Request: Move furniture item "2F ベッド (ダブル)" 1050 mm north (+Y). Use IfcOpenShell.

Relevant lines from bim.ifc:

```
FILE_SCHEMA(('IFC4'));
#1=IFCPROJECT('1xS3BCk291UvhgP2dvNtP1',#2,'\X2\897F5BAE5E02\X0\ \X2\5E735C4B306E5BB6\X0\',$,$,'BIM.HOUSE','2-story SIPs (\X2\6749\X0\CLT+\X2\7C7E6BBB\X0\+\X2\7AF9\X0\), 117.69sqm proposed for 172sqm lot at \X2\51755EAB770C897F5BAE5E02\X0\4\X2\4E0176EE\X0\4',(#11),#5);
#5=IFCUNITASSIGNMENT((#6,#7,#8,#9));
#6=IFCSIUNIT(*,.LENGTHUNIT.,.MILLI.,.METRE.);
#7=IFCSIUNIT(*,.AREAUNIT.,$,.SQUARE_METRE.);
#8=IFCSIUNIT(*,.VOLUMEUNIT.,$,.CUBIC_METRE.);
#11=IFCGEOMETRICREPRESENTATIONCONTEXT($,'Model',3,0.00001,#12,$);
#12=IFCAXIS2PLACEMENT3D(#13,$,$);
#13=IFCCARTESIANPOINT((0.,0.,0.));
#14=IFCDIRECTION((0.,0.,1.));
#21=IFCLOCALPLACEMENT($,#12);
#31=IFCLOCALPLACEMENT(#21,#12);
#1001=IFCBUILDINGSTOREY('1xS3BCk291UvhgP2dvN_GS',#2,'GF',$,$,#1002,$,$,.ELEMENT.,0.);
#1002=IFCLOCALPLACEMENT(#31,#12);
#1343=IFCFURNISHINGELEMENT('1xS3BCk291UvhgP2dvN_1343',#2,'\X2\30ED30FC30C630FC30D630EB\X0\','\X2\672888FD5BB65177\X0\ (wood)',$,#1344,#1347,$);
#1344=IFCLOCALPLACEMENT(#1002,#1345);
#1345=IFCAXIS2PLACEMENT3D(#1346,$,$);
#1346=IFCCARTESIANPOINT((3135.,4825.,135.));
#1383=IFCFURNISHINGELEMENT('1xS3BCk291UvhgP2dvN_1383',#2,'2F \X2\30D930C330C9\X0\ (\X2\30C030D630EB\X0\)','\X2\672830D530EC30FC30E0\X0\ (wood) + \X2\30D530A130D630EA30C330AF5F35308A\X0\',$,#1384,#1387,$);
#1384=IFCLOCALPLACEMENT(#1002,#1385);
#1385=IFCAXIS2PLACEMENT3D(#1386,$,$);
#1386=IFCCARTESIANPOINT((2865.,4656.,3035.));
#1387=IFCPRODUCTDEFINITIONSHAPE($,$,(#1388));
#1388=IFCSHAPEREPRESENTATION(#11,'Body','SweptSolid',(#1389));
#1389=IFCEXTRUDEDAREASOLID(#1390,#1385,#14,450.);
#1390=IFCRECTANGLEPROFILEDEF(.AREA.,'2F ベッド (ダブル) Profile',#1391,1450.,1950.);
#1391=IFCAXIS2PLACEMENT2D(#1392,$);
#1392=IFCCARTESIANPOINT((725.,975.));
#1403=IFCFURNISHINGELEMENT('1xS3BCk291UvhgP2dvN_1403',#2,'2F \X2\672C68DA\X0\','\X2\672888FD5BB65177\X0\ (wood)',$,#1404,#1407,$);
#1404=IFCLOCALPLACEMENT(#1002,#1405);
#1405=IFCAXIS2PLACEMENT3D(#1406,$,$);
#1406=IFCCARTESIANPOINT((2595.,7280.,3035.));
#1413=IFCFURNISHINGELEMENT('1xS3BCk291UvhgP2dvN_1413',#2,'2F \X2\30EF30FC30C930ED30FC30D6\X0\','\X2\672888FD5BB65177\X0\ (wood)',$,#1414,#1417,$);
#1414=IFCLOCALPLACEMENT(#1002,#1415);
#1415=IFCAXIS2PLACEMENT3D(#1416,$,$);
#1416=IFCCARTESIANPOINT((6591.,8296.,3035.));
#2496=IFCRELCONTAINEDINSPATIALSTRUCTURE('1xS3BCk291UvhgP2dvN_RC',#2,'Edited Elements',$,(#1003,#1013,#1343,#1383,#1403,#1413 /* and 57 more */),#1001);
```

```python
import ifcopenshell
import ifcopenshell.api.geometry
import ifcopenshell.util.placement
import ifcopenshell.util.unit

model = ifcopenshell.open("bim.ifc")
unit_scale = ifcopenshell.util.unit.calculate_unit_scale(model)

item = model.by_id(1383)
matrix = ifcopenshell.util.placement.get_local_placement(item.ObjectPlacement)
matrix[1, 3] += 1.05 / unit_scale
ifcopenshell.api.geometry.edit_object_placement(model, product=item, matrix=matrix, is_si=False)

print(ifcopenshell.util.placement.get_local_placement(item.ObjectPlacement).round(3) + 0.0)

model.write("bim_updated.ifc")
```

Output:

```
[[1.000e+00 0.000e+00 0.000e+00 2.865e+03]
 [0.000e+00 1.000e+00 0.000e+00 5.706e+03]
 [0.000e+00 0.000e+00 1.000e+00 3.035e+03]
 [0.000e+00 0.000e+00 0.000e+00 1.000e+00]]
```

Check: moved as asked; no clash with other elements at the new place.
